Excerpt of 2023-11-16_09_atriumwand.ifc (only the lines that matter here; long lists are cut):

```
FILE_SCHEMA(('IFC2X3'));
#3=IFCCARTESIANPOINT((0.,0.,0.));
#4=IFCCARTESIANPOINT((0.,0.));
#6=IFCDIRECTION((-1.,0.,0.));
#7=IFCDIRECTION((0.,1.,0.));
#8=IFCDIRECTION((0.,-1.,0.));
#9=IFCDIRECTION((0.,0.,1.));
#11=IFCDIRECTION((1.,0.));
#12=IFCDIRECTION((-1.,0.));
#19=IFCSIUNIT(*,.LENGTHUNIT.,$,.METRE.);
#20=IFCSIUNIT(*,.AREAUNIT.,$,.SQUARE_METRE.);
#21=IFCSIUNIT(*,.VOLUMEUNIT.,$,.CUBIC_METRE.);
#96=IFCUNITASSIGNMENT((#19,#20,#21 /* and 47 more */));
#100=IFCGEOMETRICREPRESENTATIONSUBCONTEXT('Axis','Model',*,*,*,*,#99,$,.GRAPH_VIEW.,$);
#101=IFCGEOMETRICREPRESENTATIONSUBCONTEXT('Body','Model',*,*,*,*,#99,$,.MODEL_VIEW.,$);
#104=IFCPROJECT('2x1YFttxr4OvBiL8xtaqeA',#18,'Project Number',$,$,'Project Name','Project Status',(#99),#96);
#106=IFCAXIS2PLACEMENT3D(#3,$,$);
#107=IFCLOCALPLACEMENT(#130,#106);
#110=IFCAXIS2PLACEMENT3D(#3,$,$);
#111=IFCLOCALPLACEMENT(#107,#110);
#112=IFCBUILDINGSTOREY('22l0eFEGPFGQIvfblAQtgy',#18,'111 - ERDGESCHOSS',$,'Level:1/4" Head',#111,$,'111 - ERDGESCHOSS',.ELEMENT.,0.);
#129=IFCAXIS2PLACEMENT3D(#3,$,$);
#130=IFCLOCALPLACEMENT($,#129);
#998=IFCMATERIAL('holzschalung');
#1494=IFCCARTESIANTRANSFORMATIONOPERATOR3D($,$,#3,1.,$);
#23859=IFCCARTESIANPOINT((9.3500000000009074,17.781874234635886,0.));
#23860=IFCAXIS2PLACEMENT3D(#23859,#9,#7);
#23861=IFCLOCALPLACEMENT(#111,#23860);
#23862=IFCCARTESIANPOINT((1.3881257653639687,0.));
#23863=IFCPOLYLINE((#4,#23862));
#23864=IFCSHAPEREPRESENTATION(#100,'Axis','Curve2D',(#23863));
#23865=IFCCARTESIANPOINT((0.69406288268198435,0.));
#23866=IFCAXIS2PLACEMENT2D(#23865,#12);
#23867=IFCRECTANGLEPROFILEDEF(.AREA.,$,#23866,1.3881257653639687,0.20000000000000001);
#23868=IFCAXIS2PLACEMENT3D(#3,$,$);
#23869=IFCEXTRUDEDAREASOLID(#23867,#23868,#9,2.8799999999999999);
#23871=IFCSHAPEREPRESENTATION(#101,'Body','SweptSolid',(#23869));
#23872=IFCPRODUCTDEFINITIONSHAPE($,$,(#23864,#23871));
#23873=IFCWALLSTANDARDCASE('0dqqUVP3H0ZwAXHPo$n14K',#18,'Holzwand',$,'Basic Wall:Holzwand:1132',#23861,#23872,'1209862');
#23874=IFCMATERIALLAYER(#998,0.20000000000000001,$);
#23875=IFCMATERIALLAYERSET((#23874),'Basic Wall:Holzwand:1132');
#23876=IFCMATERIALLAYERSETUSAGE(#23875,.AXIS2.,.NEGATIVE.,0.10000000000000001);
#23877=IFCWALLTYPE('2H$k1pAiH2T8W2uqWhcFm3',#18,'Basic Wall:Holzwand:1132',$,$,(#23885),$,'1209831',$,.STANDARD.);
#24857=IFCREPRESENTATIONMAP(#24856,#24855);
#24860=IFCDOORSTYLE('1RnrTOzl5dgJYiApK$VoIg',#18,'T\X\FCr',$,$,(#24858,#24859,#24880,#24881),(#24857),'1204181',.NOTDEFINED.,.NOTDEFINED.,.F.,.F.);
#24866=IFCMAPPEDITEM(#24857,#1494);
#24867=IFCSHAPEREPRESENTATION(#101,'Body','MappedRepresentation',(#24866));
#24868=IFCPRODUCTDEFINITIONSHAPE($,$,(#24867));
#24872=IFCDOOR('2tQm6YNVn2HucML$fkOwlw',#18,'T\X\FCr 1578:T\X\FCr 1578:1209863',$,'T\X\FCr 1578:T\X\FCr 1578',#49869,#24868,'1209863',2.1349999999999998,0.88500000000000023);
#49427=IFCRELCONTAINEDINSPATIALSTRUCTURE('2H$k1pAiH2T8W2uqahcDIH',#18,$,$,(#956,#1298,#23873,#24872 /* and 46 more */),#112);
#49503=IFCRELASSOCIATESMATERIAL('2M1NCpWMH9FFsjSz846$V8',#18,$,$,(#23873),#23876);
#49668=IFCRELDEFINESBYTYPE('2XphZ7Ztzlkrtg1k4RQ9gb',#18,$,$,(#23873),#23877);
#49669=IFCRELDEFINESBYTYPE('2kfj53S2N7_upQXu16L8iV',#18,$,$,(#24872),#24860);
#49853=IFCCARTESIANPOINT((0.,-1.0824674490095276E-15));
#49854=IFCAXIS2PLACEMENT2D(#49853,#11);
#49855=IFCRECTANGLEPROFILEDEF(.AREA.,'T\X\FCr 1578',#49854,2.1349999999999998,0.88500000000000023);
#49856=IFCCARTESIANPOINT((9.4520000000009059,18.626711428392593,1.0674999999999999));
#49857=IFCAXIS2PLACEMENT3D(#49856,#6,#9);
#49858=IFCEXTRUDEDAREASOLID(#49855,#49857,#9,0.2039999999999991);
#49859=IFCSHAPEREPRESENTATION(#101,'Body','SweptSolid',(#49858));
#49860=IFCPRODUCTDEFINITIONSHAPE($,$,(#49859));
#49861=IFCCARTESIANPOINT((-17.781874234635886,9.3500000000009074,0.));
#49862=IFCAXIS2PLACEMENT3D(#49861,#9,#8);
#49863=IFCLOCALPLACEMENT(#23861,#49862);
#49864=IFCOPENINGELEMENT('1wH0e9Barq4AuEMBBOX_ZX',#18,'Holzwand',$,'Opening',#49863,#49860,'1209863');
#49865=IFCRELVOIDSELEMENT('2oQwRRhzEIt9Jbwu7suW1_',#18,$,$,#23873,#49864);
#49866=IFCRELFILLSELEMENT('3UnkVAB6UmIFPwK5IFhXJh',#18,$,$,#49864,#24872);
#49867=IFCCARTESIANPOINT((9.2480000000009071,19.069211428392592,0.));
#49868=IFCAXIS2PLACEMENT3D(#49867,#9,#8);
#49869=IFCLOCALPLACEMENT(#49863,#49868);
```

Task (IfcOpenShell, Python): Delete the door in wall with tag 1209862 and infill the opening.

```python
import ifcopenshell
import ifcopenshell.api.feature
import ifcopenshell.api.root
import ifcopenshell.geom
import ifcopenshell.util.shape

model = ifcopenshell.open("2023-11-16_09_atriumwand.ifc")
settings = ifcopenshell.geom.settings()


def volume(element):
    """Net volume in cubic metres, openings subtracted."""
    shape = ifcopenshell.geom.create_shape(settings, element)
    return ifcopenshell.util.shape.get_volume(shape.geometry)


door = model.by_id(24872)
opening = door.FillsVoids[0].RelatingOpeningElement
wall = opening.VoidsElements[0].RelatingBuildingElement
before = volume(wall)

ifcopenshell.api.root.remove_product(model, product=door)
ifcopenshell.api.feature.remove_feature(model, feature=opening)

after = volume(wall)

print(f"wall volume {before:.3f} -> {after:.3f} m3")

model.write("2023-11-16_09_atriumwand-out.ifc")
```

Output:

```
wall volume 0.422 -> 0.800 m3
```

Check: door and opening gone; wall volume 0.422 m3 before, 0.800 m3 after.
